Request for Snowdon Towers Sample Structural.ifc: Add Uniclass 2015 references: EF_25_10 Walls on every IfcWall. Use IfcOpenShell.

First a look at what the model holds.

```python
import ifcopenshell

model = ifcopenshell.open("Snowdon Towers Sample Structural.ifc")
print(model.schema)
print("classifications:", [c.Name for c in model.by_type("IfcClassification")])
for ifc_class in ("IfcDoor", "IfcRoof", "IfcStair", "IfcWall", "IfcWindow"):
    print(ifc_class, len(model.by_type(ifc_class)))
```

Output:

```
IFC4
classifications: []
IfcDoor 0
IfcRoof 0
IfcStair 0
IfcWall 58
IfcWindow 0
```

```python
import ifcopenshell
import ifcopenshell.api.classification

model = ifcopenshell.open("Snowdon Towers Sample Structural.ifc")

system = ifcopenshell.api.classification.add_classification(model, classification="Uniclass 2015")

codes = {
    "IfcWall": ("EF_25_10", "Walls"),
}
for ifc_class, (code, name) in codes.items():
    products = model.by_type(ifc_class)
    ifcopenshell.api.classification.add_reference(
        model, products=products, classification=system, identification=code, name=name
    )
    print(code, len(products))

model.write("Snowdon Towers Sample Structural_edited.ifc")
```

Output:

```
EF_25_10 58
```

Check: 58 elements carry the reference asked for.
